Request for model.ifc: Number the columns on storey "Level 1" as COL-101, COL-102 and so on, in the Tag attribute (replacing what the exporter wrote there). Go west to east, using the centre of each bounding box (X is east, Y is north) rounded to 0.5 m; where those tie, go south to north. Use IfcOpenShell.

First a look at what the model holds.

```python
import ifcopenshell
import ifcopenshell.util.element
import ifcopenshell.util.placement

model = ifcopenshell.open("model.ifc")
print(model.schema)
storey = next(s for s in model.by_type("IfcBuildingStorey") if s.Name == "Level 1")
columns = [e for e in ifcopenshell.util.element.get_decomposition(storey) if e.is_a("IfcColumn")]
for e in sorted(columns, key=lambda e: e.id()):
    origin = ifcopenshell.util.placement.get_local_placement(e.ObjectPlacement)[:3, 3]
    print(e.id(), e.Tag, e.Name, origin.round(2) + 0.0, sep=" | ")
```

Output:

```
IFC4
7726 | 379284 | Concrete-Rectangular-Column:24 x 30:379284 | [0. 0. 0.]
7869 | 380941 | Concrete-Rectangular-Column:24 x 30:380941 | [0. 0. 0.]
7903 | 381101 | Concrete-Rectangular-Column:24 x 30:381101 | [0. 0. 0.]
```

```python
import ifcopenshell
import ifcopenshell.geom
import ifcopenshell.util.element
import ifcopenshell.util.shape

model = ifcopenshell.open("model.ifc")
settings = ifcopenshell.geom.settings()
settings.set("use-world-coords", True)


def centre(element):
    shape = ifcopenshell.geom.create_shape(settings, element)
    return ifcopenshell.util.shape.get_bbox_centroid(shape.geometry)


storey = next(s for s in model.by_type("IfcBuildingStorey") if s.Name == "Level 1")
columns = [e for e in ifcopenshell.util.element.get_decomposition(storey) if e.is_a("IfcColumn")]

# Insertion points can sit at a corner or the storey origin, so sort by the geometry (in metres).
centres = {e: centre(e) for e in columns}
columns.sort(key=lambda e: (round(centres[e][0] / 0.5), centres[e][1]))

for i, e in enumerate(columns, start=1):
    number = f"COL-1{i:02d}"
    e.Tag = number
    print(e.id(), number)

model.write("model-out.ifc")
```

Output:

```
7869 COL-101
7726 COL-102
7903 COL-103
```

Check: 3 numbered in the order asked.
